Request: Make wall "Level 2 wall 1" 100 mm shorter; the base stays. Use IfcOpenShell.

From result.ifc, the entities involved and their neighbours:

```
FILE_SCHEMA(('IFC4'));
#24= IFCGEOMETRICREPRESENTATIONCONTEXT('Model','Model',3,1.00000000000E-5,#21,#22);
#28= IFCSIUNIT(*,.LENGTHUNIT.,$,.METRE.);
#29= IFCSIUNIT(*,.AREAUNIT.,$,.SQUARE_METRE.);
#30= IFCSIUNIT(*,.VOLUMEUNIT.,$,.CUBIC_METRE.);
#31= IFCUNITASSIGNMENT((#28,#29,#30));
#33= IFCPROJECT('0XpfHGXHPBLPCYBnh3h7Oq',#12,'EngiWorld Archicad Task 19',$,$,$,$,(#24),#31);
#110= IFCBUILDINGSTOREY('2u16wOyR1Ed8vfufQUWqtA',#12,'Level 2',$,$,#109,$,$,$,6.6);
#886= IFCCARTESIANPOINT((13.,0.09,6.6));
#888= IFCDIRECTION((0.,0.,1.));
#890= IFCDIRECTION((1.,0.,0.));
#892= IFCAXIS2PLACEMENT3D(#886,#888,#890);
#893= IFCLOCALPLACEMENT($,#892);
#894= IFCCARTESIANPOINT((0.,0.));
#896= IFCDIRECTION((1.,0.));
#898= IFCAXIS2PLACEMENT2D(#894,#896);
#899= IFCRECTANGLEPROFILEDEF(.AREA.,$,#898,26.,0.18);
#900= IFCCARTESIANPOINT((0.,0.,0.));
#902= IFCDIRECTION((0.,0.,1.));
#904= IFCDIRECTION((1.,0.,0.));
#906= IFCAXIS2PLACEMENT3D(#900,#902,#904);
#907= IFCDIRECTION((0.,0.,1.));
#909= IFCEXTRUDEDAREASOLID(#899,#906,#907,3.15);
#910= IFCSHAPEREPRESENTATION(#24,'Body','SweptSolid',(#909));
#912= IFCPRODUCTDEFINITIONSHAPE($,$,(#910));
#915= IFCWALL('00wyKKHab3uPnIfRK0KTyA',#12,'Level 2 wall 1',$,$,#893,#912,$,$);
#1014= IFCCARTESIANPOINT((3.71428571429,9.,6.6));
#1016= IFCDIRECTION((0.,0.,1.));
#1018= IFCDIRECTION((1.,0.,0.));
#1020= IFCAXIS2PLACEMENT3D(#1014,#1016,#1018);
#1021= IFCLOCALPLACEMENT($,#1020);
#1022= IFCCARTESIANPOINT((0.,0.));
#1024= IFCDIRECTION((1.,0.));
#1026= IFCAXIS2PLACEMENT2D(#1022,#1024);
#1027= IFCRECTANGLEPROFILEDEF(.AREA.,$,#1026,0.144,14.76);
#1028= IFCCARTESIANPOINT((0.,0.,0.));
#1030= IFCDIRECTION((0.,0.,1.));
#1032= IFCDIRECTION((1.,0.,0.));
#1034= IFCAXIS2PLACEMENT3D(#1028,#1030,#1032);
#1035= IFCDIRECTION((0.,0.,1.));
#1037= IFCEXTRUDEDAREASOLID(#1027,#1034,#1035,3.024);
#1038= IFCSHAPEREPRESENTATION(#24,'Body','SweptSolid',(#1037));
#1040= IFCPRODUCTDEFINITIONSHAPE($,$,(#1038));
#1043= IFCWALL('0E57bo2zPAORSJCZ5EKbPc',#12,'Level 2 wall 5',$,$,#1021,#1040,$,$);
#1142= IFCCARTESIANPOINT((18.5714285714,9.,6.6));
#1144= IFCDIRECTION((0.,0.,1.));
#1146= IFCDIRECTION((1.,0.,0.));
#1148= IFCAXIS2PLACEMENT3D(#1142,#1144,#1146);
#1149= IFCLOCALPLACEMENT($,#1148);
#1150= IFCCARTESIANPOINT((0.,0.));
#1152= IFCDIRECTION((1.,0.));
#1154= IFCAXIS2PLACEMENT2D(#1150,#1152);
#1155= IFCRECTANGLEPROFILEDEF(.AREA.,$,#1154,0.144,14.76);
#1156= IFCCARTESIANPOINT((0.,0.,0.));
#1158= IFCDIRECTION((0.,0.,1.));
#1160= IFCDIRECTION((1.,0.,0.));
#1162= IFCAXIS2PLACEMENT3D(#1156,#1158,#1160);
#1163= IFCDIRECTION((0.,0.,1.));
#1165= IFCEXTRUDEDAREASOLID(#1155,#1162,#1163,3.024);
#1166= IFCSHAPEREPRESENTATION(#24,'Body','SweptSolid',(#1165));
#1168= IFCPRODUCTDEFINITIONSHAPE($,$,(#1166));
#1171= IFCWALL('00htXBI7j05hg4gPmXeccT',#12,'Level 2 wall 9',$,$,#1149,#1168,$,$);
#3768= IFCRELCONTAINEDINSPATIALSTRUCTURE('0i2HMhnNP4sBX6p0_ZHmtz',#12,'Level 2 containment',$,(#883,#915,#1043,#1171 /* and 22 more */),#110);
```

```python
import ifcopenshell
import ifcopenshell.geom
import ifcopenshell.util.shape
import ifcopenshell.util.unit

model = ifcopenshell.open("result.ifc")
unit_scale = ifcopenshell.util.unit.calculate_unit_scale(model)
settings = ifcopenshell.geom.settings()


def volume(element):
    """Net volume in cubic metres, openings subtracted."""
    shape = ifcopenshell.geom.create_shape(settings, element)
    return ifcopenshell.util.shape.get_volume(shape.geometry)


wall = model.by_guid("00wyKKHab3uPnIfRK0KTyA")
before = volume(wall)

body = next(r for r in wall.Representation.Representations if r.RepresentationIdentifier == "Body")
solid = body.Items[0]
old_height = solid.Depth
solid.Depth -= 0.1 / unit_scale
after = volume(wall)

print(f"height {old_height:g} -> {solid.Depth:g}, volume {before:.3f} -> {after:.3f} m3")

model.write("result_v2.ifc")
```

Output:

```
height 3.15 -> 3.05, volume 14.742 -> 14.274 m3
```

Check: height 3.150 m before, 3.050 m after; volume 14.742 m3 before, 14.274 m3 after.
